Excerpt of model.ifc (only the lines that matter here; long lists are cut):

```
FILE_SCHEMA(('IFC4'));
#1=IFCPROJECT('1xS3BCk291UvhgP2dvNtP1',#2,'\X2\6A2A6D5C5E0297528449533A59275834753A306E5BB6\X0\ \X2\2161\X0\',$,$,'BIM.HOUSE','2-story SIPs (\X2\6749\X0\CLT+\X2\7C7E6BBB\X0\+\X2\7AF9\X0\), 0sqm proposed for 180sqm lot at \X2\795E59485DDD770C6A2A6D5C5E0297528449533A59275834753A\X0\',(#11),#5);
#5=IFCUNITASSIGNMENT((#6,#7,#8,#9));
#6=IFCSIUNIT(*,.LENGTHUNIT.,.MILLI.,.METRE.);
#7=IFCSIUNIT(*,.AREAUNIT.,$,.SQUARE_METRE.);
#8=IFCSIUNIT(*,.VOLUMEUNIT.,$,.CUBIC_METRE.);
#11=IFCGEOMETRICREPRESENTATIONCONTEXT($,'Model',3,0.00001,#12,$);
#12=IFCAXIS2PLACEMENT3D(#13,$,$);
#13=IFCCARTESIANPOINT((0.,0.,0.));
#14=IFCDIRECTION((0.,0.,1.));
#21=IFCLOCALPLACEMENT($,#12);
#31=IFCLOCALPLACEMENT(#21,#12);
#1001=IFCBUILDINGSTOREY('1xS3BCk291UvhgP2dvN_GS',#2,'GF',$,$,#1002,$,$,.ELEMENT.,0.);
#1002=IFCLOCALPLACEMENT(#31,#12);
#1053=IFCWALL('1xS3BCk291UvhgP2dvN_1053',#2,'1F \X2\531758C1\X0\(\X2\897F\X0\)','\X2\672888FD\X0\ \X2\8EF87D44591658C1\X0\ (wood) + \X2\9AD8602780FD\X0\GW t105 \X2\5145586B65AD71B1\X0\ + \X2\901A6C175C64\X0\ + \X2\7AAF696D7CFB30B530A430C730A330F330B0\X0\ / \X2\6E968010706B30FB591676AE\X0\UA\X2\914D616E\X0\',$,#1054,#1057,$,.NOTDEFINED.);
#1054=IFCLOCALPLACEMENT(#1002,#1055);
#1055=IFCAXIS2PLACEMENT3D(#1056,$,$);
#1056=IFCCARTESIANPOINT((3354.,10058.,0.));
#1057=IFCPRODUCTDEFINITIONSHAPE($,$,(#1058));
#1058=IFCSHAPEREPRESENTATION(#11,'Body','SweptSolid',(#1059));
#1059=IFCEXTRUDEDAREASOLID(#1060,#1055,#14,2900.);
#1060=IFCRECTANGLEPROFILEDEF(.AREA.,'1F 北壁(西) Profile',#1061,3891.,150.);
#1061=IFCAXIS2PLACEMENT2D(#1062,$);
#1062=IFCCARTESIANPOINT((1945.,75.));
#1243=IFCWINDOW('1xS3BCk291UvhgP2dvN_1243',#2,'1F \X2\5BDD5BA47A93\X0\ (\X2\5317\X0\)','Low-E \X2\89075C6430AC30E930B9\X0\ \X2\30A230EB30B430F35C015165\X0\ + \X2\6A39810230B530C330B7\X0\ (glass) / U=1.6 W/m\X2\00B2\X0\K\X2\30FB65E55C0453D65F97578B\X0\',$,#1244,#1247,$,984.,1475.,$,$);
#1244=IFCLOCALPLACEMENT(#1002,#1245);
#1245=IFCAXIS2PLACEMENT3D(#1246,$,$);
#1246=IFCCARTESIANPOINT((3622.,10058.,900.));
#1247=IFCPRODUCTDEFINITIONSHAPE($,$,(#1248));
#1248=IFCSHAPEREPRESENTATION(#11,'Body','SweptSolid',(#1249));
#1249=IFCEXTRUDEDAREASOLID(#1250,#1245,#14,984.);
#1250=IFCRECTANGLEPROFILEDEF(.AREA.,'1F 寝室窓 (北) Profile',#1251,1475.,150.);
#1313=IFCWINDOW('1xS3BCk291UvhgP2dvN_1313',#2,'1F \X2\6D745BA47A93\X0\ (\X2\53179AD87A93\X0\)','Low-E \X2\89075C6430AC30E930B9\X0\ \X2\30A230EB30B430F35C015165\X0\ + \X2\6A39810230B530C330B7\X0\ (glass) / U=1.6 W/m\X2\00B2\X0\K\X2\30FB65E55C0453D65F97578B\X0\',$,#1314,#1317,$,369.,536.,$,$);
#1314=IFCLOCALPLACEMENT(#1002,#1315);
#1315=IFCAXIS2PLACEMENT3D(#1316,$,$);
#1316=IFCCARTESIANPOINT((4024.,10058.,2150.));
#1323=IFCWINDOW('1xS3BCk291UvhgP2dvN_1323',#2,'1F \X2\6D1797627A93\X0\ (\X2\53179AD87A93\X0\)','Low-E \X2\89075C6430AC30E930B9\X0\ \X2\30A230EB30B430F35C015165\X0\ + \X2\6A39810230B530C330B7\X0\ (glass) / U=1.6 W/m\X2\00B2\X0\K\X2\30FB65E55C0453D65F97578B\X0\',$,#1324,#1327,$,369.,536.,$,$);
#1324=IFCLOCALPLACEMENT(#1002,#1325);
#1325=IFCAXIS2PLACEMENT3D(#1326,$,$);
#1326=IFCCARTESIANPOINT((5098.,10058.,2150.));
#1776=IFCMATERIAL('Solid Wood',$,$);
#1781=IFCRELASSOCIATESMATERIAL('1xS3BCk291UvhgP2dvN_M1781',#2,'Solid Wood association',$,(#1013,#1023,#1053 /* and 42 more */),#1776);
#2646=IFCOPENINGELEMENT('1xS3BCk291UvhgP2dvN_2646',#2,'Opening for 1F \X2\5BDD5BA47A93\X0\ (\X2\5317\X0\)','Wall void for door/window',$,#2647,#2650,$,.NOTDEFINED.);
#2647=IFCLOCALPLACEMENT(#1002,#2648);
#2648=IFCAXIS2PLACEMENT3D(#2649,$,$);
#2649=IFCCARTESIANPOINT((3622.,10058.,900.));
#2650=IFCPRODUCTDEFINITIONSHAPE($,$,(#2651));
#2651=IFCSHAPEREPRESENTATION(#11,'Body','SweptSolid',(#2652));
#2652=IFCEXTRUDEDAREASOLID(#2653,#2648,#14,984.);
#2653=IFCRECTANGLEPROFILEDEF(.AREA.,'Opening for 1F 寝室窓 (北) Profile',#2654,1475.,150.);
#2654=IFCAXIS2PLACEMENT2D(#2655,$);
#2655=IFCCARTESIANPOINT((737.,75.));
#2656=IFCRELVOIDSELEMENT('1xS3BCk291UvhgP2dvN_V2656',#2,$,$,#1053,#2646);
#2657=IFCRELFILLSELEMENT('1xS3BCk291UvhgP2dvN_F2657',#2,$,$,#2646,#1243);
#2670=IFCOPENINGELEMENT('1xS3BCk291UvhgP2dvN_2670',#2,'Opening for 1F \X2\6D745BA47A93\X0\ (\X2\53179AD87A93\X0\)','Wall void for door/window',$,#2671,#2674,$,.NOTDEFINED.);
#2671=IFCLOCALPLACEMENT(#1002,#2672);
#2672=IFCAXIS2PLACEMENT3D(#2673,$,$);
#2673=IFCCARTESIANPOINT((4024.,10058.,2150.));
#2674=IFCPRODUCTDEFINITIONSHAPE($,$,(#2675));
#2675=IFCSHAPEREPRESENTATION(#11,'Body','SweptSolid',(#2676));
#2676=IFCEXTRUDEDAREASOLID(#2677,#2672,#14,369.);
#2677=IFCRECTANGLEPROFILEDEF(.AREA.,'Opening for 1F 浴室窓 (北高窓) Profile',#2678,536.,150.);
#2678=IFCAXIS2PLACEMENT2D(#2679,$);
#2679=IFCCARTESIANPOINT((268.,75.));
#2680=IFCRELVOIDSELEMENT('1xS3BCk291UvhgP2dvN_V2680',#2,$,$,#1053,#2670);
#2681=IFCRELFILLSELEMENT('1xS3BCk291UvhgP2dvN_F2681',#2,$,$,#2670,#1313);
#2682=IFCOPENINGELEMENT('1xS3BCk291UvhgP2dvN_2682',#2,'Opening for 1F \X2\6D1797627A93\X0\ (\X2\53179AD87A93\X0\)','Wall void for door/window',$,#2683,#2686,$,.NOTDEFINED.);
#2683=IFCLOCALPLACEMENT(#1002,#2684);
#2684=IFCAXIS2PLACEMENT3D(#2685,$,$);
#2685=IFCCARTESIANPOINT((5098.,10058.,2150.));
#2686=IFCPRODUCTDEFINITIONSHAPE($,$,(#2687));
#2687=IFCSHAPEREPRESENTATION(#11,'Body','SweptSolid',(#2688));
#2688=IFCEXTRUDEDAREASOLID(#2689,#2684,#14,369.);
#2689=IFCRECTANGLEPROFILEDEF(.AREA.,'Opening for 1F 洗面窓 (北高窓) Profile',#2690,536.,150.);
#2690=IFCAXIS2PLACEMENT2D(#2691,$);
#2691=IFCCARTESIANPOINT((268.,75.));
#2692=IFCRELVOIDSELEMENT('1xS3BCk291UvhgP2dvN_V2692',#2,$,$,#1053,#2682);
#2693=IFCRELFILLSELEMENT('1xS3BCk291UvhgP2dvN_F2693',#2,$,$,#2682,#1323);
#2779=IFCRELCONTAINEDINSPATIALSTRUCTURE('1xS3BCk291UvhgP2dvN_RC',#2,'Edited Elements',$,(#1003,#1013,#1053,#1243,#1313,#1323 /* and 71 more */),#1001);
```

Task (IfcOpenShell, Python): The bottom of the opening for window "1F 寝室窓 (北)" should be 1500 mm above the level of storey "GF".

```python
import numpy as np
import ifcopenshell
import ifcopenshell.api.geometry
import ifcopenshell.geom
import ifcopenshell.util.element
import ifcopenshell.util.placement
import ifcopenshell.util.shape
import ifcopenshell.util.unit

model = ifcopenshell.open("model.ifc")
unit_scale = ifcopenshell.util.unit.calculate_unit_scale(model)

window = model.by_guid("1xS3BCk291UvhgP2dvN_1243")
opening = window.FillsVoids[0].RelatingOpeningElement
storey = ifcopenshell.util.element.get_container(window, ifc_class="IfcBuildingStorey")
level = ifcopenshell.util.placement.get_local_placement(storey.ObjectPlacement)[2, 3]

# The opening's origin need not be at the sill, so measure its lowest point.
shape = ifcopenshell.geom.create_shape(ifcopenshell.geom.settings(), opening)
bottom = ifcopenshell.util.shape.get_shape_bottom_elevation(shape, shape.geometry) / unit_scale
dz = level + 1.5 / unit_scale - bottom

shift = np.array([0.0, 0.0, dz])
# The window is not placed relative to its opening, so move both.
for product in (opening, window):
    matrix = ifcopenshell.util.placement.get_local_placement(product.ObjectPlacement)
    matrix[:3, 3] += shift
    ifcopenshell.api.geometry.edit_object_placement(model, product=product, matrix=matrix, is_si=False)

print(f"moved by {dz * unit_scale:+.3f} m")

model.write("model_rev.ifc")
```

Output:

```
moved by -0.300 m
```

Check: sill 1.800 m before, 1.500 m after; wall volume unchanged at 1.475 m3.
